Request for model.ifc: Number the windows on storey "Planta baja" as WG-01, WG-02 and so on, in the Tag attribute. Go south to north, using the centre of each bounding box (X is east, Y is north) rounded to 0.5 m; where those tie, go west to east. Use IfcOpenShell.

First a look at what the model holds.

```python
import ifcopenshell
import ifcopenshell.util.element
import ifcopenshell.util.placement

model = ifcopenshell.open("model.ifc")
print(model.schema)
storey = next(s for s in model.by_type("IfcBuildingStorey") if s.Name == "Planta baja")
windows = [e for e in ifcopenshell.util.element.get_decomposition(storey) if e.is_a("IfcWindow")]
for e in sorted(windows, key=lambda e: e.id()):
    origin = ifcopenshell.util.placement.get_local_placement(e.ObjectPlacement)[:3, 3]
    print(e.id(), e.Tag, e.Name, origin.round(2) + 0.0, sep=" | ")
```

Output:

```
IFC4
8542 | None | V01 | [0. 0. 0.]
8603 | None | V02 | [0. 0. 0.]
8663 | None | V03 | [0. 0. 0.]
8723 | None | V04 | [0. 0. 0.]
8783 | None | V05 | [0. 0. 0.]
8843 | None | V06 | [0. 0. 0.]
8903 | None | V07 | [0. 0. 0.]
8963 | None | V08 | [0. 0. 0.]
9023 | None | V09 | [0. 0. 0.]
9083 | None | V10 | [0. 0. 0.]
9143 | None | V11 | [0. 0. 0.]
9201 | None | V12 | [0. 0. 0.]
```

```python
import ifcopenshell
import ifcopenshell.geom
import ifcopenshell.util.element
import ifcopenshell.util.shape

model = ifcopenshell.open("model.ifc")
settings = ifcopenshell.geom.settings()
settings.set("use-world-coords", True)


def centre(element):
    shape = ifcopenshell.geom.create_shape(settings, element)
    return ifcopenshell.util.shape.get_bbox_centroid(shape.geometry)


storey = next(s for s in model.by_type("IfcBuildingStorey") if s.Name == "Planta baja")
windows = [e for e in ifcopenshell.util.element.get_decomposition(storey) if e.is_a("IfcWindow")]

# Insertion points can sit at a corner or the storey origin, so sort by the geometry (in metres).
centres = {e: centre(e) for e in windows}
windows.sort(key=lambda e: (round(centres[e][1] / 0.5), centres[e][0]))

for i, e in enumerate(windows, start=1):
    number = f"WG-{i:02d}"
    e.Tag = number
    print(e.id(), number)

model.write("model_edited.ifc")
```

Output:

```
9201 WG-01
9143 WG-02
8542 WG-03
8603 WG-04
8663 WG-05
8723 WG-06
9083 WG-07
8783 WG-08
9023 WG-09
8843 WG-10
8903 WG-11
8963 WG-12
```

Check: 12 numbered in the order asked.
